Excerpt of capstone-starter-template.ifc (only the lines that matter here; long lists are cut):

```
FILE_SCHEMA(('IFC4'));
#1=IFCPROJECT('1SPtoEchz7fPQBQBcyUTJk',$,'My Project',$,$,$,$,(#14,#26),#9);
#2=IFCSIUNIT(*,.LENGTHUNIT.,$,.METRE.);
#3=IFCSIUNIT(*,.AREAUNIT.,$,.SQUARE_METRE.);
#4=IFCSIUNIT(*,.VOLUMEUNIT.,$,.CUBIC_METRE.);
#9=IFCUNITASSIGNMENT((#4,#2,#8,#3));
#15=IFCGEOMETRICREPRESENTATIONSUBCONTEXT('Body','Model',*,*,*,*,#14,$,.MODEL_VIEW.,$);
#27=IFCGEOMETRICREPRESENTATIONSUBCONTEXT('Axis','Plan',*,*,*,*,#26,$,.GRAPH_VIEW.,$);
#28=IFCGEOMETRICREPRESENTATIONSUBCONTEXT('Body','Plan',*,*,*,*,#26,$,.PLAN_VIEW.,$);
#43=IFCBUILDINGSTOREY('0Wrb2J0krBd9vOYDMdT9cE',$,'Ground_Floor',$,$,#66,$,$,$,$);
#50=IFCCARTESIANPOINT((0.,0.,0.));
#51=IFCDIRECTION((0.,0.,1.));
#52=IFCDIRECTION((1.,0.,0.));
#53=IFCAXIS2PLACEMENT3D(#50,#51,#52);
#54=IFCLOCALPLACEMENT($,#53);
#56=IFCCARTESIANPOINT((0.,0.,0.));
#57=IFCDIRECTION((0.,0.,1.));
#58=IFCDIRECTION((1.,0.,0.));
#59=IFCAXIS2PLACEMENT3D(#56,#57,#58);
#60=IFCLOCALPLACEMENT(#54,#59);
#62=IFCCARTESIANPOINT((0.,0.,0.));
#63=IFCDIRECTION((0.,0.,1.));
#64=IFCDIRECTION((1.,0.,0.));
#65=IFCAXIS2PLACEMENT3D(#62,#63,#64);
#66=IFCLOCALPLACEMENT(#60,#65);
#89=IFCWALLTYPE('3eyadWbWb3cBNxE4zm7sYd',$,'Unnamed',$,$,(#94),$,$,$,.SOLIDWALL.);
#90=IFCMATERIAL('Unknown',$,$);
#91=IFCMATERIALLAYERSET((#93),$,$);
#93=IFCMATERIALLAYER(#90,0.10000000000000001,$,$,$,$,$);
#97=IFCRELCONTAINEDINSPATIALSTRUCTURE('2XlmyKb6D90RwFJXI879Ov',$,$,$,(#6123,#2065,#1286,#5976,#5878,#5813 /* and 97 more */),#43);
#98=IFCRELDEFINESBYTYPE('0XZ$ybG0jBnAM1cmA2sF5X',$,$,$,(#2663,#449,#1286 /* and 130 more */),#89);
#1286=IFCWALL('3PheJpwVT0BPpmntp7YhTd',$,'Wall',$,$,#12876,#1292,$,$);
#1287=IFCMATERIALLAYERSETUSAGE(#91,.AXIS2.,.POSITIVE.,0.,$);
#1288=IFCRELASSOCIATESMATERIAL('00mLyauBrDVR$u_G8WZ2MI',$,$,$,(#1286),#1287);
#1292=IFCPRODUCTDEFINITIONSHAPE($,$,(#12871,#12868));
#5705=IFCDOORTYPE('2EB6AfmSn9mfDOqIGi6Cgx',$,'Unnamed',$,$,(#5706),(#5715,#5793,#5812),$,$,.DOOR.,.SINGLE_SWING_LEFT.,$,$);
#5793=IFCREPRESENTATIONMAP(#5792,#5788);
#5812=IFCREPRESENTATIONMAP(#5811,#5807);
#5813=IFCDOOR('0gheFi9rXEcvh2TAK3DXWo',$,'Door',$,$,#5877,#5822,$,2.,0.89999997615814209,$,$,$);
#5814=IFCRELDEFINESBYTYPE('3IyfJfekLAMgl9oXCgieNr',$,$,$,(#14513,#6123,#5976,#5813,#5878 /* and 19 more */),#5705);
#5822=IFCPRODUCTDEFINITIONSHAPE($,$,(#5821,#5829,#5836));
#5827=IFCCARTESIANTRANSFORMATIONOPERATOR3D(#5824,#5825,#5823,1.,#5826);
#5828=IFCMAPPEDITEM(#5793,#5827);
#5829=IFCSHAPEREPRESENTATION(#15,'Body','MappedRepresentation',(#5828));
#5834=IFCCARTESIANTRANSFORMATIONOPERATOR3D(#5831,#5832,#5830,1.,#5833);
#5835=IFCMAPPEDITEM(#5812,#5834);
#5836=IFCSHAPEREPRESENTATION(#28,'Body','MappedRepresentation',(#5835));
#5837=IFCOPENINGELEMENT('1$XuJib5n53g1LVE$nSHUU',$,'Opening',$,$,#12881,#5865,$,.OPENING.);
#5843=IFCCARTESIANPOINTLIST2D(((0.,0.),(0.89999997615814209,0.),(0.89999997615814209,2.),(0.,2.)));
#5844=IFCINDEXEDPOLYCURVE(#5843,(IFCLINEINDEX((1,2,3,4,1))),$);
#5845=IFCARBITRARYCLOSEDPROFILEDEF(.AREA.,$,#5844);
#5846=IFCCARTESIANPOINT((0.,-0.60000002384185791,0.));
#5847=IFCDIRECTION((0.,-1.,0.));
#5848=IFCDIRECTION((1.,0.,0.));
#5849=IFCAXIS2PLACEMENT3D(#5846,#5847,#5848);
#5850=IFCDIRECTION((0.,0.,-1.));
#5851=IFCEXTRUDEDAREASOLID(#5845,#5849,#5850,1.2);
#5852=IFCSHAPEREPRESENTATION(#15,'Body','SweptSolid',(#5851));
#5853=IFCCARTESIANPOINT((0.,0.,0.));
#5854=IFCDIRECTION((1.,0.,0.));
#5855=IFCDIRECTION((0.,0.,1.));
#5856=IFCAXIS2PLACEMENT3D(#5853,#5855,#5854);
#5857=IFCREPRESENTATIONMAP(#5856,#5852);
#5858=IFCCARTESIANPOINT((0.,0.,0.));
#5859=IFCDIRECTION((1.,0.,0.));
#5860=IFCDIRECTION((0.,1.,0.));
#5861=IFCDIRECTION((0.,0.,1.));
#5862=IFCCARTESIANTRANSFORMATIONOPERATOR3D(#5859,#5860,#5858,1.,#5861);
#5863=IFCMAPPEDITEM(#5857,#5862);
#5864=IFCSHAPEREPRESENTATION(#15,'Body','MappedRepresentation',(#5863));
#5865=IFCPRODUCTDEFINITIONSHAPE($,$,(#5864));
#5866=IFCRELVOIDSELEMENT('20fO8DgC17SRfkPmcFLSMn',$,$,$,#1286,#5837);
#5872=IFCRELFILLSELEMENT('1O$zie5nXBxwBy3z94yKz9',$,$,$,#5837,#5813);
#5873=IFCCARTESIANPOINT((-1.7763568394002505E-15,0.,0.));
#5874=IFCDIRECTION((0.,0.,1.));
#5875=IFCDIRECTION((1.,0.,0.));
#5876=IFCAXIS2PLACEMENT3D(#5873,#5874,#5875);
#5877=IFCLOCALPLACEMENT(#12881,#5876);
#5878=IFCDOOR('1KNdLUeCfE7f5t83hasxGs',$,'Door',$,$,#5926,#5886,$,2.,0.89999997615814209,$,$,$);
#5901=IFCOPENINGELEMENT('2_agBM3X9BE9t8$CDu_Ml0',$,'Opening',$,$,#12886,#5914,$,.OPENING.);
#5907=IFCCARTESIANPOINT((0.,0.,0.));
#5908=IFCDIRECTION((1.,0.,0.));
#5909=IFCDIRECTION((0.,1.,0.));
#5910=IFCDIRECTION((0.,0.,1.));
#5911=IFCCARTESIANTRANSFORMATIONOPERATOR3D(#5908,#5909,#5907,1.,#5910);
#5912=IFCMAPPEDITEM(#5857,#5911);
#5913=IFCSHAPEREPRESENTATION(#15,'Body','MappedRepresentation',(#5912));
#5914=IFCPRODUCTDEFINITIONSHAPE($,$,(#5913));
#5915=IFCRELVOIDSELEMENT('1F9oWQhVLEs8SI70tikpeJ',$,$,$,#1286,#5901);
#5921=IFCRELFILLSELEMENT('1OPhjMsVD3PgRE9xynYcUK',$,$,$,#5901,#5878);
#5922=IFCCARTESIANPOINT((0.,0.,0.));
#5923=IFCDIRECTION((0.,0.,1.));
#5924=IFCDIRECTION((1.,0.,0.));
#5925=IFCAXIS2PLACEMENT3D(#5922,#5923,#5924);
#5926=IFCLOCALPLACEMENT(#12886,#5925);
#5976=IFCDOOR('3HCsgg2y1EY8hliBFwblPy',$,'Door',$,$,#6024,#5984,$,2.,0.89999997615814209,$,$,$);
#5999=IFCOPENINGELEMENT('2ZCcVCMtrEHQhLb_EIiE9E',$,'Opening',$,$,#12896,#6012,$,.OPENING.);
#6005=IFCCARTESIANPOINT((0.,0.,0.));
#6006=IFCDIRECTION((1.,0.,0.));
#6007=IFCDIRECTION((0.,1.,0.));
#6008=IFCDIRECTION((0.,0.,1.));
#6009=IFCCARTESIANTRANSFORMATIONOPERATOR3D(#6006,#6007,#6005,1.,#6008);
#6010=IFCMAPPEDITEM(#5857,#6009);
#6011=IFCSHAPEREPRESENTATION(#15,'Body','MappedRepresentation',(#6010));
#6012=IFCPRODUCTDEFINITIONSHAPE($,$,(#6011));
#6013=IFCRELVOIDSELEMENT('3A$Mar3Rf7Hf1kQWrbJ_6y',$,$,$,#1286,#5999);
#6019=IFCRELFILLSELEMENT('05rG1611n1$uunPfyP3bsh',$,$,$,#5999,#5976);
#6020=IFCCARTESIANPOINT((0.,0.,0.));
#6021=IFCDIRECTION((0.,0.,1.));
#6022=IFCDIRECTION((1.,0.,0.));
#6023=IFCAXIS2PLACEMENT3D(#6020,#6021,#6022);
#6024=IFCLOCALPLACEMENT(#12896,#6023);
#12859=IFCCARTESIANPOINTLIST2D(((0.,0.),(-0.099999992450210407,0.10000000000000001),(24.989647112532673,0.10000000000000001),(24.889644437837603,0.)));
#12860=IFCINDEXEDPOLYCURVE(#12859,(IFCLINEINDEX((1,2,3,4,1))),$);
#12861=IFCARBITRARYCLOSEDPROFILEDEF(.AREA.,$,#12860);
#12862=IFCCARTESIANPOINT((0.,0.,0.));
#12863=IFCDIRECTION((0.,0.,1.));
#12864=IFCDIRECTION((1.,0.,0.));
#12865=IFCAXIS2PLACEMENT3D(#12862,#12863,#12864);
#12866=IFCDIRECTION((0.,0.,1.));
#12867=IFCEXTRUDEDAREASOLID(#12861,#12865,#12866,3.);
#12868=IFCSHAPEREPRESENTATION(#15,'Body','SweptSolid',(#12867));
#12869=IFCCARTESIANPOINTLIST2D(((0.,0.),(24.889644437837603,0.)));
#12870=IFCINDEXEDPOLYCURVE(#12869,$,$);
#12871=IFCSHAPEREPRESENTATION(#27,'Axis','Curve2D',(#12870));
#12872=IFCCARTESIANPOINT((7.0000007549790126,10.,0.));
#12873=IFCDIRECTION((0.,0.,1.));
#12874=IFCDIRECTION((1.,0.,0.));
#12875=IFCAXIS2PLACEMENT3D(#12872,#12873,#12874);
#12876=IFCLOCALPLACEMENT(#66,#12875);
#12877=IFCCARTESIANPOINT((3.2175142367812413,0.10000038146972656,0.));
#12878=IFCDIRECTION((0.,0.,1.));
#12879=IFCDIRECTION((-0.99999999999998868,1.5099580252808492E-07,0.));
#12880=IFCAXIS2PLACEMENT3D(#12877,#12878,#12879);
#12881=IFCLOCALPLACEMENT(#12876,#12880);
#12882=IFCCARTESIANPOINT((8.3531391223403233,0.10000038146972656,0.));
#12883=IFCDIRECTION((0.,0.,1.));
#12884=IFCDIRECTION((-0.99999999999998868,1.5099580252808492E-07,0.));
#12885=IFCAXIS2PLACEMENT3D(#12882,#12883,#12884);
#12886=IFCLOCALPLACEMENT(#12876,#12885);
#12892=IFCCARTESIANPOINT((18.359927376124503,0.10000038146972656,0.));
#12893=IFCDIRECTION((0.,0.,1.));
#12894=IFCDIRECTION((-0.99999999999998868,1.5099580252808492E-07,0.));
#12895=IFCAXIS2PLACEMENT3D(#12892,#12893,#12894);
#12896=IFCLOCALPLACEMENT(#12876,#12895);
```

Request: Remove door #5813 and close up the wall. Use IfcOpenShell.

```python
import ifcopenshell
import ifcopenshell.api.feature
import ifcopenshell.api.root
import ifcopenshell.geom
import ifcopenshell.util.shape

model = ifcopenshell.open("capstone-starter-template.ifc")
settings = ifcopenshell.geom.settings()


def volume(element):
    """Net volume in cubic metres, openings subtracted."""
    shape = ifcopenshell.geom.create_shape(settings, element)
    return ifcopenshell.util.shape.get_volume(shape.geometry)


door = model.by_id(5813)
opening = door.FillsVoids[0].RelatingOpeningElement
wall = opening.VoidsElements[0].RelatingBuildingElement
before = volume(wall)

ifcopenshell.api.root.remove_product(model, product=door)
ifcopenshell.api.feature.remove_feature(model, feature=opening)

after = volume(wall)

print(f"wall volume {before:.3f} -> {after:.3f} m3")

model.write("capstone-starter-template_updated.ifc")
```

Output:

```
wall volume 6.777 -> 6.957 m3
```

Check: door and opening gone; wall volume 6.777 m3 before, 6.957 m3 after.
